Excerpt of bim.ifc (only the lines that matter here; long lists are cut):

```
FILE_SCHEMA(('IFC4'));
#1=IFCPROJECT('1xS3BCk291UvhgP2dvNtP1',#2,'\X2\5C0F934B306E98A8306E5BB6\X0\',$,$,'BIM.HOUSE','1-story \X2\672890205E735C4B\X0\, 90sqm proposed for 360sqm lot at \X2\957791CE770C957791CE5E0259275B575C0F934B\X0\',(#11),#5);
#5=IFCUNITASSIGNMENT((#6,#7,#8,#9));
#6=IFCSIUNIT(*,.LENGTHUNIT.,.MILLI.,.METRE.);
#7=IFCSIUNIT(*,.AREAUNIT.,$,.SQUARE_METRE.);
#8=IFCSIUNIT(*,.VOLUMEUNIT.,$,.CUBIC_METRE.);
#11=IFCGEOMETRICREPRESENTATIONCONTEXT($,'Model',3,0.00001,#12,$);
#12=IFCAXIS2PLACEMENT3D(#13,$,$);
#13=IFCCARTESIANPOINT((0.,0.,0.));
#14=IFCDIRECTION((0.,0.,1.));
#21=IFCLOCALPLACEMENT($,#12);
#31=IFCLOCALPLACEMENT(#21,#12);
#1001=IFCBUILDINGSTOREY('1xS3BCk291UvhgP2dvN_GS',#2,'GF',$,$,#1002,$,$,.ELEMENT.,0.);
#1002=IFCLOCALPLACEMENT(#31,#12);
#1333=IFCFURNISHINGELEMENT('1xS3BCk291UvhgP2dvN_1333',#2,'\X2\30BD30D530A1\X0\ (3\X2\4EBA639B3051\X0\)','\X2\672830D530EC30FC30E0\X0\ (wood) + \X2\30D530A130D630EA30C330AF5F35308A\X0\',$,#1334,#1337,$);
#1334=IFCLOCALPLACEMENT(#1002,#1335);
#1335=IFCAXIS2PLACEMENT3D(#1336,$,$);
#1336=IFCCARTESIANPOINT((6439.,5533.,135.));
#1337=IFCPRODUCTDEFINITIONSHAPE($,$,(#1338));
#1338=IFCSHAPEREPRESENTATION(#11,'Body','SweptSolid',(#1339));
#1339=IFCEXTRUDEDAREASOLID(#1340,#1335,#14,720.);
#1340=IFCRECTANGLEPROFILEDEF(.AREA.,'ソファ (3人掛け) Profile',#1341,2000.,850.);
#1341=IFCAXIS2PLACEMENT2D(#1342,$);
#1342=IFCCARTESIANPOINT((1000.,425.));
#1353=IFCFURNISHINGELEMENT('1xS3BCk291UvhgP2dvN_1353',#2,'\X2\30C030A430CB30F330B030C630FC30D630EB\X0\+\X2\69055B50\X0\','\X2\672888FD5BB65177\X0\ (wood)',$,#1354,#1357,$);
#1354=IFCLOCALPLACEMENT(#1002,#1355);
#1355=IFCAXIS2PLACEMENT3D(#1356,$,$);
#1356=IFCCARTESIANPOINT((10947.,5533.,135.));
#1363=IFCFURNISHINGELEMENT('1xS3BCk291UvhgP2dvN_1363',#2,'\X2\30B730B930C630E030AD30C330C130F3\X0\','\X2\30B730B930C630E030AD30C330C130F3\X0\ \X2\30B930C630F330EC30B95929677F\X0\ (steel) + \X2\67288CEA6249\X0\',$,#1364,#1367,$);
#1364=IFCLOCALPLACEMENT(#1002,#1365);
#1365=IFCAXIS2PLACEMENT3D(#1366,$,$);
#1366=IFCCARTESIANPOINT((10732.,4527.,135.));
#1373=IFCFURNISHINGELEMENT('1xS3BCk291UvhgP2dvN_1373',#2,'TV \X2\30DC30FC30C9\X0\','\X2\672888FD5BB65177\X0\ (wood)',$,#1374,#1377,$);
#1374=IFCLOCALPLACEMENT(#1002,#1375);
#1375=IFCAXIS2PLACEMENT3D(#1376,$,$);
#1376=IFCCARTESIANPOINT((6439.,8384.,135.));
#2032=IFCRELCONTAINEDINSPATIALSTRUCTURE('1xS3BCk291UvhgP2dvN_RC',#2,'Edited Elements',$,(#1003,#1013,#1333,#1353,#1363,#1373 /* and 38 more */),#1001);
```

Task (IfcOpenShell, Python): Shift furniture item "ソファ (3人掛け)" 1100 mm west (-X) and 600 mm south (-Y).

```python
import ifcopenshell
import ifcopenshell.api.geometry
import ifcopenshell.util.placement

model = ifcopenshell.open("bim.ifc")

item = model.by_id(1333)
matrix = ifcopenshell.util.placement.get_local_placement(item.ObjectPlacement)
matrix[0, 3] -= 1100.0
matrix[1, 3] -= 600.0
ifcopenshell.api.geometry.edit_object_placement(model, product=item, matrix=matrix, is_si=False)

print(ifcopenshell.util.placement.get_local_placement(item.ObjectPlacement).round(3) + 0.0)

model.write("bim_updated.ifc")
```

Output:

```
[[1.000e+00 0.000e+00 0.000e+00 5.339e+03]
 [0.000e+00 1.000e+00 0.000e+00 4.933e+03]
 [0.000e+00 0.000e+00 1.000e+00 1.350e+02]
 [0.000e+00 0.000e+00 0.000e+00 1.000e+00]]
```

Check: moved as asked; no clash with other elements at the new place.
